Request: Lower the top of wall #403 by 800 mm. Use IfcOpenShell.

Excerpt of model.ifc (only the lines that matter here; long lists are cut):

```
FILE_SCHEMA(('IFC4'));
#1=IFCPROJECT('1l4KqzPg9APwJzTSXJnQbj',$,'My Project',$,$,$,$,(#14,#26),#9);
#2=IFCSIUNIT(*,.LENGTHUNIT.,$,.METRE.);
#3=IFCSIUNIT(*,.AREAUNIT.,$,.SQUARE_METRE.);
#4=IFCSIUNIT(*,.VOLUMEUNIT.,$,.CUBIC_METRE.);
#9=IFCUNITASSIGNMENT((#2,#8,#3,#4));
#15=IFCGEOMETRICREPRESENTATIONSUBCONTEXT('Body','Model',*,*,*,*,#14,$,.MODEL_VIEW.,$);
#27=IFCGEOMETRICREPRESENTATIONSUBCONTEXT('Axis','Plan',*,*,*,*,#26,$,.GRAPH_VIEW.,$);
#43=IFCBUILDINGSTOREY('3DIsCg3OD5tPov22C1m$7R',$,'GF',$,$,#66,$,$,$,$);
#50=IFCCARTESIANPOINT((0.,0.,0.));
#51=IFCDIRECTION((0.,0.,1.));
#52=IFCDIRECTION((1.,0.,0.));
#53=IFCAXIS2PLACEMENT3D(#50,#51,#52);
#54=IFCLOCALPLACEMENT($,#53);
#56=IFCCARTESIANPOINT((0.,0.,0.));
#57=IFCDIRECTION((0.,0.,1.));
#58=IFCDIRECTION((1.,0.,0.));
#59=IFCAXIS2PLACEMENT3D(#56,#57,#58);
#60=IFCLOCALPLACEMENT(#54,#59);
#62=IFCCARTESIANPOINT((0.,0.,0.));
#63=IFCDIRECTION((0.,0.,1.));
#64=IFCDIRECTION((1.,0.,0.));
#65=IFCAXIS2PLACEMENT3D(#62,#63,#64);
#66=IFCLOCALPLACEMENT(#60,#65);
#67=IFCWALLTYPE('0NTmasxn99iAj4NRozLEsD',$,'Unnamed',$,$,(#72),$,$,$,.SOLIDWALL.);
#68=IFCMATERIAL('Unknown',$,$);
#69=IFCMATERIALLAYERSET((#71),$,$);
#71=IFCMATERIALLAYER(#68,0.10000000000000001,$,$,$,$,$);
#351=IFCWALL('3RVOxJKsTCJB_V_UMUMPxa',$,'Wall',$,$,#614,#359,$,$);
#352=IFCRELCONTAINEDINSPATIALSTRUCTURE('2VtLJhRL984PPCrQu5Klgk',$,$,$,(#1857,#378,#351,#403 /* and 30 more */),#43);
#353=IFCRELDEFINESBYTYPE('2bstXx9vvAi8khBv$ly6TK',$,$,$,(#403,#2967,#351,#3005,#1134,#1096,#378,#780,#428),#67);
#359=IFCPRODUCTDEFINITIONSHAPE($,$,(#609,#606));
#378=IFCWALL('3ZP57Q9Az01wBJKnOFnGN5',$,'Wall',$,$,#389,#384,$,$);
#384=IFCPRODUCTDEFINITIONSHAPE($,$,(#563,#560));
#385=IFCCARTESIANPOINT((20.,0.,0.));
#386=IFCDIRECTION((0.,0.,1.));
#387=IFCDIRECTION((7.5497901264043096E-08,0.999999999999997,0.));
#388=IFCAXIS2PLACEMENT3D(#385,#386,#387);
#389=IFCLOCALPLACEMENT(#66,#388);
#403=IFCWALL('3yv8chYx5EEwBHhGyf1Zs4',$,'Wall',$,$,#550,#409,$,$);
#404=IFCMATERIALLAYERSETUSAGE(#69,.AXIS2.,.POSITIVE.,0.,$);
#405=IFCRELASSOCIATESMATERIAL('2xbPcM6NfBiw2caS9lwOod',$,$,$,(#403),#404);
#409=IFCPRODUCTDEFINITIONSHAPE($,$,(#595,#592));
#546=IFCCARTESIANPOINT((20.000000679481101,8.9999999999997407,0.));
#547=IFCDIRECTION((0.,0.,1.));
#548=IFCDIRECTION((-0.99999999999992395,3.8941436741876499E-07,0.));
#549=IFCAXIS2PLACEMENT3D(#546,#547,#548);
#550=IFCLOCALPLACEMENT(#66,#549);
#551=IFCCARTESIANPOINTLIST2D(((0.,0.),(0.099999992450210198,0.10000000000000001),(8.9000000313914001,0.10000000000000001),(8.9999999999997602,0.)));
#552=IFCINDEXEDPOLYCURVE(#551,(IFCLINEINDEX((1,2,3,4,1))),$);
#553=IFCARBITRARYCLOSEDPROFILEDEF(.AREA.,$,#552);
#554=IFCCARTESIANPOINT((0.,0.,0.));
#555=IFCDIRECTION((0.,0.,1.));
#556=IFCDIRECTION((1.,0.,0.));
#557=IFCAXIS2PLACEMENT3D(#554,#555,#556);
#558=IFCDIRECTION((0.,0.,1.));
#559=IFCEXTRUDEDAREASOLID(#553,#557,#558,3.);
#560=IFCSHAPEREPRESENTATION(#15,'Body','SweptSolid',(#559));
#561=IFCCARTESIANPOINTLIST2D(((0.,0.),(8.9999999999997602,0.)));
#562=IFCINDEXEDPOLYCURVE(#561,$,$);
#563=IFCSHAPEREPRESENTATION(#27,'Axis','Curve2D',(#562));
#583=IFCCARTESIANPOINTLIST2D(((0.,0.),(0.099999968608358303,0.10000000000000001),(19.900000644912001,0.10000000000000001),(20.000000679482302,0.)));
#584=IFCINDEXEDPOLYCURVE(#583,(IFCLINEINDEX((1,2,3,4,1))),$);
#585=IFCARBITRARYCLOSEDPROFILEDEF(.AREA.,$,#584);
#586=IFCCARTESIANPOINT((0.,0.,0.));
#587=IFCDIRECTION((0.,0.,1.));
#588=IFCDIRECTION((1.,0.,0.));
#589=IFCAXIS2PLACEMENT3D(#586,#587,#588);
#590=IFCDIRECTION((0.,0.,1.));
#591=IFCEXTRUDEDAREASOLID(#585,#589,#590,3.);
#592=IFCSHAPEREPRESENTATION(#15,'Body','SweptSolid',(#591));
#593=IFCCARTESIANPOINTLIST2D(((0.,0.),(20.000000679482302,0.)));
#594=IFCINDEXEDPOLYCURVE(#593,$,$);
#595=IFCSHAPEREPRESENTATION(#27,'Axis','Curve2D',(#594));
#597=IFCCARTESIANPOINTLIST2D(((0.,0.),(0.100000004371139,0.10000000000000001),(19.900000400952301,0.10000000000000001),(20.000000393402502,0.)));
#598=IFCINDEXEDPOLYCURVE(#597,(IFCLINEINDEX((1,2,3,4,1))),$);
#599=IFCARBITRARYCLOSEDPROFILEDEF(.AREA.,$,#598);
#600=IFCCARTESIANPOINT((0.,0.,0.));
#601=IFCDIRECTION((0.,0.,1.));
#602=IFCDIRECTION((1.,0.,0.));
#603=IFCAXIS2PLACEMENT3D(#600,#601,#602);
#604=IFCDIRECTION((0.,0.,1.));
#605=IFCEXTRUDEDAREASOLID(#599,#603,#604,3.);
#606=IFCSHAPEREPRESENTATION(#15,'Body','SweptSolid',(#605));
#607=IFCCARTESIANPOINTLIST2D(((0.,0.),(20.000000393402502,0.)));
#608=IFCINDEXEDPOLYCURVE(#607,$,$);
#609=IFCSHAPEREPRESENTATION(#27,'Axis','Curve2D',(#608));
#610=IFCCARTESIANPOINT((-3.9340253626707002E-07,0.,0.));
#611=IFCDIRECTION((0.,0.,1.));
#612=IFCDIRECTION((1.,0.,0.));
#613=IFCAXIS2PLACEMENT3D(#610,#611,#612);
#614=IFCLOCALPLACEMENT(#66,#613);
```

```python
import ifcopenshell
import ifcopenshell.geom
import ifcopenshell.util.representation
import ifcopenshell.util.shape
import ifcopenshell.util.unit

model = ifcopenshell.open("model.ifc")
unit_scale = ifcopenshell.util.unit.calculate_unit_scale(model)
settings = ifcopenshell.geom.settings()


def volume(element):
    """Net volume in cubic metres, openings subtracted."""
    shape = ifcopenshell.geom.create_shape(settings, element)
    return ifcopenshell.util.shape.get_volume(shape.geometry)


wall = model.by_guid("3yv8chYx5EEwBHhGyf1Zs4")
before = volume(wall)

body = ifcopenshell.util.representation.get_representation(wall, "Model", "Body")
solid = body.Items[0]
old_height = solid.Depth
solid.Depth -= 0.8 / unit_scale
after = volume(wall)

print(f"height {old_height:g} -> {solid.Depth:g}, volume {before:.3f} -> {after:.3f} m3")

model.write("model_rev.ifc")
```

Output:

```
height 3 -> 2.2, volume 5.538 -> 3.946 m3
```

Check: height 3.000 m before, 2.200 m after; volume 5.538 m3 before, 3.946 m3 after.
